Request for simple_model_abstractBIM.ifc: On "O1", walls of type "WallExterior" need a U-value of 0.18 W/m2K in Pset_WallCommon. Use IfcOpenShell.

First a look at what the model holds.

```python
import ifcopenshell
import ifcopenshell.util.element

model = ifcopenshell.open("simple_model_abstractBIM.ifc")
print(model.schema)
storey = next(s for s in model.by_type("IfcBuildingStorey") if s.Name == "O1")
walls = [e for e in ifcopenshell.util.element.get_decomposition(storey) if e.is_a("IfcWall")]
seen = {}
for e in walls:
    element_type = ifcopenshell.util.element.get_type(e)
    key = (element_type.Name if element_type != e and element_type else None, ifcopenshell.util.element.get_pset(e, "Pset_WallCommon", "ThermalTransmittance"))
    seen[key] = seen.get(key, 0) + 1
for (name, value), count in sorted(seen.items(), key=str):
    print(count, "x", name, "|", value)
```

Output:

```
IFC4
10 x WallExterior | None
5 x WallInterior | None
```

```python
import ifcopenshell
import ifcopenshell.api.pset
import ifcopenshell.util.element

model = ifcopenshell.open("simple_model_abstractBIM.ifc")

storey = next(s for s in model.by_type("IfcBuildingStorey") if s.Name == "O1")
walls = [e for e in ifcopenshell.util.element.get_decomposition(storey) if e.is_a("IfcWall")]

count = 0
for e in walls:
    element_type = ifcopenshell.util.element.get_type(e)
    if element_type in (None, e) or element_type.Name != "WallExterior":
        continue
    # add_pset returns the element's existing set when there is one.
    pset = ifcopenshell.api.pset.add_pset(model, product=e, name="Pset_WallCommon")
    ifcopenshell.api.pset.edit_pset(model, pset=pset, properties={"ThermalTransmittance": 0.18})
    count += 1

print(count, "walls updated")

model.write("simple_model_abstractBIM_rev.ifc")
```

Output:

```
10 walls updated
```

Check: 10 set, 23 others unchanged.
